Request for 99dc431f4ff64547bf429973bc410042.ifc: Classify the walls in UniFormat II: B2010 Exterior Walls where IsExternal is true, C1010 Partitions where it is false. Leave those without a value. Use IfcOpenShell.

First a look at what the model holds.

```python
import ifcopenshell
import ifcopenshell.util.element

model = ifcopenshell.open("99dc431f4ff64547bf429973bc410042.ifc")
print(model.schema)
print("classifications:", [c.Name for c in model.by_type("IfcClassification")])
values = [ifcopenshell.util.element.get_pset(e, "Pset_WallCommon", "IsExternal") for e in model.by_type("IfcWall")]
for value in (True, False, None):
    print("IsExternal", value, values.count(value))
```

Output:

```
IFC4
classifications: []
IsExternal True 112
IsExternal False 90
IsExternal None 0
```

```python
import ifcopenshell
import ifcopenshell.api.classification
import ifcopenshell.util.element

model = ifcopenshell.open("99dc431f4ff64547bf429973bc410042.ifc")

system = ifcopenshell.api.classification.add_classification(model, classification="UniFormat II")

walls = model.by_type("IfcWall")
external = {e: ifcopenshell.util.element.get_pset(e, "Pset_WallCommon", "IsExternal") for e in walls}
for flag, code, name in ((True, "B2010", "Exterior Walls"), (False, "C1010", "Partitions")):
    products = [e for e in walls if external[e] is flag]
    ifcopenshell.api.classification.add_reference(
        model, products=products, classification=system, identification=code, name=name
    )
    print(code, len(products))

model.write("99dc431f4ff64547bf429973bc410042_updated.ifc")
```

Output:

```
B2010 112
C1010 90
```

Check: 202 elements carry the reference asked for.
